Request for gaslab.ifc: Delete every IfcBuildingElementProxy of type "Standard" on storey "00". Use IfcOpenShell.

First a look at what the model holds.

```python
import ifcopenshell
import ifcopenshell.util.element

model = ifcopenshell.open("gaslab.ifc")
print(model.schema)
storey = next(s for s in model.by_type("IfcBuildingStorey") if s.Name == "00")
proxies = [e for e in ifcopenshell.util.element.get_decomposition(storey) if e.is_a("IfcBuildingElementProxy")]
seen = {}
for e in proxies:
    element_type = ifcopenshell.util.element.get_type(e)
    name = element_type.Name if element_type not in (None, e) else None
    seen[name] = seen.get(name, 0) + 1
for name, count in sorted(seen.items(), key=str):
    print(count, "x", name)
```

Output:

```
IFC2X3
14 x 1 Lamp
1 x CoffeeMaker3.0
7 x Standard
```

```python
import ifcopenshell
import ifcopenshell.api.root
import ifcopenshell.util.element

model = ifcopenshell.open("gaslab.ifc")

storey = next(s for s in model.by_type("IfcBuildingStorey") if s.Name == "00")
proxies = [e for e in ifcopenshell.util.element.get_decomposition(storey) if e.is_a("IfcBuildingElementProxy")]
targets = [e for e in proxies if (t := ifcopenshell.util.element.get_type(e)) not in (None, e) and t.Name == "Standard"]

for e in targets:
    ifcopenshell.api.root.remove_product(model, product=e)
print(len(targets), "removed")

model.write("gaslab_rev.ifc")
```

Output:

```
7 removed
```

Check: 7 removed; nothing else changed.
